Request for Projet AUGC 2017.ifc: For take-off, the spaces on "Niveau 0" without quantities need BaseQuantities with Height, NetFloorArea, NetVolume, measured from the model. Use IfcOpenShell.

First a look at what the model holds.

```python
import ifcopenshell
import ifcopenshell.util.element
import ifcopenshell.util.unit

model = ifcopenshell.open("Projet AUGC 2017.ifc")
print(model.schema)
for unit_type in ("LENGTHUNIT", "AREAUNIT", "VOLUMEUNIT"):
    print(unit_type, ifcopenshell.util.unit.calculate_unit_scale(model, unit_type))
storey = next(s for s in model.by_type("IfcBuildingStorey") if s.Name == "Niveau 0")
spaces = [e for e in ifcopenshell.util.element.get_decomposition(storey) if e.is_a("IfcSpace")]
for e in sorted(spaces, key=lambda e: e.id()):
    print(e.id(), e.is_a(), e.Name, list(ifcopenshell.util.element.get_psets(e, qtos_only=True)), sep=" | ")
```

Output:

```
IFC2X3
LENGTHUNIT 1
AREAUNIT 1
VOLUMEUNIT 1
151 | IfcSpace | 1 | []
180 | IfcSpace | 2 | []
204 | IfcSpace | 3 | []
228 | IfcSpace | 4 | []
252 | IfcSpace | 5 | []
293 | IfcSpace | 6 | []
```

```python
import ifcopenshell
import ifcopenshell.api.pset
import ifcopenshell.geom
import ifcopenshell.util.element
import ifcopenshell.util.shape
import ifcopenshell.util.unit

model = ifcopenshell.open("Projet AUGC 2017.ifc")
unit_scale = ifcopenshell.util.unit.calculate_unit_scale(model)
area_scale = ifcopenshell.util.unit.calculate_unit_scale(model, "AREAUNIT")
volume_scale = ifcopenshell.util.unit.calculate_unit_scale(model, "VOLUMEUNIT")
settings = ifcopenshell.geom.settings()

storey = next(s for s in model.by_type("IfcBuildingStorey") if s.Name == "Niveau 0")
spaces = [e for e in ifcopenshell.util.element.get_decomposition(storey) if e.is_a("IfcSpace")]

for e in sorted(spaces, key=lambda e: e.id()):
    if ifcopenshell.util.element.get_psets(e, qtos_only=True, should_inherit=False):
        continue
    # Geometry comes back in metres, in the element's own axes.
    shape = ifcopenshell.geom.create_shape(settings, e)
    values = {
        "Height": ifcopenshell.util.shape.get_z(shape.geometry) / unit_scale,
        "NetFloorArea": ifcopenshell.util.shape.get_footprint_area(shape.geometry) / area_scale,
        "NetVolume": ifcopenshell.util.shape.get_volume(shape.geometry) / volume_scale,
    }
    qto = ifcopenshell.api.pset.add_qto(model, product=e, name="BaseQuantities")
    ifcopenshell.api.pset.edit_qto(model, qto=qto, properties=values)
    print(e.id(), {k: round(v, 3) for k, v in values.items()})

model.write("Projet AUGC 2017_v2.ifc")
```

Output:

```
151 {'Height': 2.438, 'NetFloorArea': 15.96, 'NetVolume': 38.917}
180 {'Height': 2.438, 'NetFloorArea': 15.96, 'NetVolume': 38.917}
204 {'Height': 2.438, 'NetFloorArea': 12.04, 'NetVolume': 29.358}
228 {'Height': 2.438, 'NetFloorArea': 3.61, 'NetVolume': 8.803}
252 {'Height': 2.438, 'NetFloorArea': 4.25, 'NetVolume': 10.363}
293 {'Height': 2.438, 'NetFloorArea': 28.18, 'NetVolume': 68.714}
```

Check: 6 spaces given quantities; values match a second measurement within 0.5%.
